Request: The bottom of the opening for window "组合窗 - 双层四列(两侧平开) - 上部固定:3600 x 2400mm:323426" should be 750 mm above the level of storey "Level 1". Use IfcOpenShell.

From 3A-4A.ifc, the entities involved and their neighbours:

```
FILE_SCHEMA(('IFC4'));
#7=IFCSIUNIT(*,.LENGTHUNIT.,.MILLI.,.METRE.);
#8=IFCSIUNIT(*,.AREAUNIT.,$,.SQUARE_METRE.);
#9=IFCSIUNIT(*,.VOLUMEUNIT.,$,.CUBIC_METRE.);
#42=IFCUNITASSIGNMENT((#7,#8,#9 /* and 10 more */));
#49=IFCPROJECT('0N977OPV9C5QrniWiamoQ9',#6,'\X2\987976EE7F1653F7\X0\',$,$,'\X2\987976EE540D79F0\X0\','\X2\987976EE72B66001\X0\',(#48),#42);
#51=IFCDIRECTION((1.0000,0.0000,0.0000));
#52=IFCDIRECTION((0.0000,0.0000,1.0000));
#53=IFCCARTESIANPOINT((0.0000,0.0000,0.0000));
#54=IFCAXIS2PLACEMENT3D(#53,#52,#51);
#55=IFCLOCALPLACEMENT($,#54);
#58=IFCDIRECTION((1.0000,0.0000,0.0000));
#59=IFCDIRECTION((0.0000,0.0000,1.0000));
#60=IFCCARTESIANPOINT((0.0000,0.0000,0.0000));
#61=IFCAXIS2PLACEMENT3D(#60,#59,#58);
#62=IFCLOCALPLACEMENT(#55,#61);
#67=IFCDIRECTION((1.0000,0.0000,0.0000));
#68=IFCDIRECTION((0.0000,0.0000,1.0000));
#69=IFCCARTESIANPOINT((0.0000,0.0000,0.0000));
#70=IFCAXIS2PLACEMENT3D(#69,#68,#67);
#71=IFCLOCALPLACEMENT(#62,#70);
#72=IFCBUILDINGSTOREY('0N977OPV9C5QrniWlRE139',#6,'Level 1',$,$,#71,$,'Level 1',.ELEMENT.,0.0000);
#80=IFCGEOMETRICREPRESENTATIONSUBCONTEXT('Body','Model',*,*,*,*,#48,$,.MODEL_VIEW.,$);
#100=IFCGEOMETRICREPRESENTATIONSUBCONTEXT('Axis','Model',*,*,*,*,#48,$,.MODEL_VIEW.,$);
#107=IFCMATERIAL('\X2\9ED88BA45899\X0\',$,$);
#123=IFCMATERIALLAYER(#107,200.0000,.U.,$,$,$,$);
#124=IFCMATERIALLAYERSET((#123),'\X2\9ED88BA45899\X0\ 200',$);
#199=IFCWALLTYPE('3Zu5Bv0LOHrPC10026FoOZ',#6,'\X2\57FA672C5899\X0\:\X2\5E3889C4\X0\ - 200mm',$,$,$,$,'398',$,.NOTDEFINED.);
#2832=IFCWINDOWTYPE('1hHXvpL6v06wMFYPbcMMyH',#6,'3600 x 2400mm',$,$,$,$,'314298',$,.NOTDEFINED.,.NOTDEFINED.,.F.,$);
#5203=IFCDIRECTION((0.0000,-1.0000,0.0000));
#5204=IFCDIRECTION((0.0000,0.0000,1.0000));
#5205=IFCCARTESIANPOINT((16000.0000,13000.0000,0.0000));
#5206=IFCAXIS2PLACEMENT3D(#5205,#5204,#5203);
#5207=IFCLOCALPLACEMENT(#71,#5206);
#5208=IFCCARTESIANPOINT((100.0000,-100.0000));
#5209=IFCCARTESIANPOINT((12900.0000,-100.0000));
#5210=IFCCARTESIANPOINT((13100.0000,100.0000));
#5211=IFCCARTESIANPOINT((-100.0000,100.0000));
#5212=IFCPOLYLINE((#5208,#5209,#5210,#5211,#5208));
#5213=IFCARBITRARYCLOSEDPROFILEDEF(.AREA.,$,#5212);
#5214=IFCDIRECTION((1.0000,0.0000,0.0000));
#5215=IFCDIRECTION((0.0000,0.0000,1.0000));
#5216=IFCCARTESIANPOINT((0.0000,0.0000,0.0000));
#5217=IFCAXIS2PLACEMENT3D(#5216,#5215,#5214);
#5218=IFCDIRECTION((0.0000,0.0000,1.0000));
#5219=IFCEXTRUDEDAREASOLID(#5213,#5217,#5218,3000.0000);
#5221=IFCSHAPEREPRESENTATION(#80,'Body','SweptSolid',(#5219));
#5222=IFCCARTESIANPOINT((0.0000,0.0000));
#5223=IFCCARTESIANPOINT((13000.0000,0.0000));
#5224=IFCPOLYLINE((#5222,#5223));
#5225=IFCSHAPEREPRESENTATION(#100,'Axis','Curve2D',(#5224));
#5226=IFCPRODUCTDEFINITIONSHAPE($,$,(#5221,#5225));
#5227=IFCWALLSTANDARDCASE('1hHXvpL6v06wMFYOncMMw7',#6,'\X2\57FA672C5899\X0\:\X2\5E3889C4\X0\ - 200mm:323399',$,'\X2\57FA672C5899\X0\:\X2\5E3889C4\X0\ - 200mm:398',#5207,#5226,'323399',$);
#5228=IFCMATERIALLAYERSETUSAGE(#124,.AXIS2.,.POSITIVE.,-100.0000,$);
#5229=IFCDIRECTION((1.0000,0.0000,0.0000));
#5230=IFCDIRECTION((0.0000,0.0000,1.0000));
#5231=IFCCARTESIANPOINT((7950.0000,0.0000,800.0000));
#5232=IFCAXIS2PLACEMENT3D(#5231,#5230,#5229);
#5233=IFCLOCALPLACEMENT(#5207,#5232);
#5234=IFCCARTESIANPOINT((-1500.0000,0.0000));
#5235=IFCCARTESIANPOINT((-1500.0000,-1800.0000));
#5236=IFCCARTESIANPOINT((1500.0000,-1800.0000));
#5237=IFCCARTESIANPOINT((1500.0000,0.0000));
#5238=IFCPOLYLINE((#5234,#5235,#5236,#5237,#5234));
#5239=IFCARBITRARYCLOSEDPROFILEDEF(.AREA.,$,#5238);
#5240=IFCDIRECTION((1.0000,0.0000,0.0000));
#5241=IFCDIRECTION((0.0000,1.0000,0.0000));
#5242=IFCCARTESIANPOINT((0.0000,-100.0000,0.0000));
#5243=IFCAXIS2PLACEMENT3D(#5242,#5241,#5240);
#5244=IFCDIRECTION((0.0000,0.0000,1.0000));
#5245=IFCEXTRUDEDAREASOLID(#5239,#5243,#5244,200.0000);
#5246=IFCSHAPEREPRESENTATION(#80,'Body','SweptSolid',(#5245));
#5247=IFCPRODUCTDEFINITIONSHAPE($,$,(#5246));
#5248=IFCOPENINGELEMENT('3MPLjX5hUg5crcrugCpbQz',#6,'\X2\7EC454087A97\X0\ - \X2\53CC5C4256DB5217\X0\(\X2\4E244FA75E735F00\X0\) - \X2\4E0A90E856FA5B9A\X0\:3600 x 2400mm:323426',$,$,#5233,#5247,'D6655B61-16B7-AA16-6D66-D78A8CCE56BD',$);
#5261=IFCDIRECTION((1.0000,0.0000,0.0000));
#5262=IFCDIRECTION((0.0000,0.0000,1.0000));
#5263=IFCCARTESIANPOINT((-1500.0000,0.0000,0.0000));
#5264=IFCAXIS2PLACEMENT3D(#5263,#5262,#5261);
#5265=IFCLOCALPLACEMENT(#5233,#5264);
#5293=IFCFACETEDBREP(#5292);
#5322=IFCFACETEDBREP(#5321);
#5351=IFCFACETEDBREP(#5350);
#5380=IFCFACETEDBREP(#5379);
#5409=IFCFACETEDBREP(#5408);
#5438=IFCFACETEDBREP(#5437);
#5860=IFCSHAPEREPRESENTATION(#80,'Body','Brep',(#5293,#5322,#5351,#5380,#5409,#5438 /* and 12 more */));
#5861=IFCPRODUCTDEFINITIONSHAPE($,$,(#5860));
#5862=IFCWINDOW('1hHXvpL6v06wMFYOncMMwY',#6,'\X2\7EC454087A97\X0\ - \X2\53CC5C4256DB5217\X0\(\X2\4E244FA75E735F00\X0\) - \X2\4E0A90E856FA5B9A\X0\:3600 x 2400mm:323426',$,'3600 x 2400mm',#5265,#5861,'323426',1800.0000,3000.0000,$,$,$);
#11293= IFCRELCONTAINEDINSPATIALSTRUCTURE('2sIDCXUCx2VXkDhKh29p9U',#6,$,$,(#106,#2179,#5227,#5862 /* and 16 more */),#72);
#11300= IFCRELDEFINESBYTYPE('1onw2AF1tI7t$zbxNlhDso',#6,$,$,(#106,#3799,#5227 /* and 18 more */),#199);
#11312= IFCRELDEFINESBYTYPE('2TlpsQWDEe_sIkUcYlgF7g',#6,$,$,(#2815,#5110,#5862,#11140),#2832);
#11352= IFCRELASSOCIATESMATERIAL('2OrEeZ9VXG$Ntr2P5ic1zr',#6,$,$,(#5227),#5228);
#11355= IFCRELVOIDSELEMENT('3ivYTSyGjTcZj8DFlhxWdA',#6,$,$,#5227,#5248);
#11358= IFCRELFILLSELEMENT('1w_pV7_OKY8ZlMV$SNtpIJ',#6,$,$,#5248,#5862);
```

```python
import numpy as np
import ifcopenshell
import ifcopenshell.api.geometry
import ifcopenshell.geom
import ifcopenshell.util.element
import ifcopenshell.util.placement
import ifcopenshell.util.shape
import ifcopenshell.util.unit

model = ifcopenshell.open("3A-4A.ifc")
unit_scale = ifcopenshell.util.unit.calculate_unit_scale(model)

window = model.by_guid("1hHXvpL6v06wMFYOncMMwY")
opening = window.FillsVoids[0].RelatingOpeningElement
storey = ifcopenshell.util.element.get_container(window, ifc_class="IfcBuildingStorey")
level = ifcopenshell.util.placement.get_local_placement(storey.ObjectPlacement)[2, 3]

# The opening's origin need not be at the sill, so measure its lowest point.
shape = ifcopenshell.geom.create_shape(ifcopenshell.geom.settings(), opening)
bottom = ifcopenshell.util.shape.get_shape_bottom_elevation(shape, shape.geometry) / unit_scale
dz = level + 0.75 / unit_scale - bottom

shift = np.array([0.0, 0.0, dz])
# The window is placed relative to its opening, so it follows when the opening moves.
matrix = ifcopenshell.util.placement.get_local_placement(opening.ObjectPlacement)
matrix[:3, 3] += shift
ifcopenshell.api.geometry.edit_object_placement(
    model, product=opening, matrix=matrix, is_si=False, should_transform_children=True
)

print(f"moved by {dz * unit_scale:+.3f} m")

model.write("3A-4A-out.ifc")
```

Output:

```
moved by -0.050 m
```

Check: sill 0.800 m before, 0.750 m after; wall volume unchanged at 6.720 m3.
